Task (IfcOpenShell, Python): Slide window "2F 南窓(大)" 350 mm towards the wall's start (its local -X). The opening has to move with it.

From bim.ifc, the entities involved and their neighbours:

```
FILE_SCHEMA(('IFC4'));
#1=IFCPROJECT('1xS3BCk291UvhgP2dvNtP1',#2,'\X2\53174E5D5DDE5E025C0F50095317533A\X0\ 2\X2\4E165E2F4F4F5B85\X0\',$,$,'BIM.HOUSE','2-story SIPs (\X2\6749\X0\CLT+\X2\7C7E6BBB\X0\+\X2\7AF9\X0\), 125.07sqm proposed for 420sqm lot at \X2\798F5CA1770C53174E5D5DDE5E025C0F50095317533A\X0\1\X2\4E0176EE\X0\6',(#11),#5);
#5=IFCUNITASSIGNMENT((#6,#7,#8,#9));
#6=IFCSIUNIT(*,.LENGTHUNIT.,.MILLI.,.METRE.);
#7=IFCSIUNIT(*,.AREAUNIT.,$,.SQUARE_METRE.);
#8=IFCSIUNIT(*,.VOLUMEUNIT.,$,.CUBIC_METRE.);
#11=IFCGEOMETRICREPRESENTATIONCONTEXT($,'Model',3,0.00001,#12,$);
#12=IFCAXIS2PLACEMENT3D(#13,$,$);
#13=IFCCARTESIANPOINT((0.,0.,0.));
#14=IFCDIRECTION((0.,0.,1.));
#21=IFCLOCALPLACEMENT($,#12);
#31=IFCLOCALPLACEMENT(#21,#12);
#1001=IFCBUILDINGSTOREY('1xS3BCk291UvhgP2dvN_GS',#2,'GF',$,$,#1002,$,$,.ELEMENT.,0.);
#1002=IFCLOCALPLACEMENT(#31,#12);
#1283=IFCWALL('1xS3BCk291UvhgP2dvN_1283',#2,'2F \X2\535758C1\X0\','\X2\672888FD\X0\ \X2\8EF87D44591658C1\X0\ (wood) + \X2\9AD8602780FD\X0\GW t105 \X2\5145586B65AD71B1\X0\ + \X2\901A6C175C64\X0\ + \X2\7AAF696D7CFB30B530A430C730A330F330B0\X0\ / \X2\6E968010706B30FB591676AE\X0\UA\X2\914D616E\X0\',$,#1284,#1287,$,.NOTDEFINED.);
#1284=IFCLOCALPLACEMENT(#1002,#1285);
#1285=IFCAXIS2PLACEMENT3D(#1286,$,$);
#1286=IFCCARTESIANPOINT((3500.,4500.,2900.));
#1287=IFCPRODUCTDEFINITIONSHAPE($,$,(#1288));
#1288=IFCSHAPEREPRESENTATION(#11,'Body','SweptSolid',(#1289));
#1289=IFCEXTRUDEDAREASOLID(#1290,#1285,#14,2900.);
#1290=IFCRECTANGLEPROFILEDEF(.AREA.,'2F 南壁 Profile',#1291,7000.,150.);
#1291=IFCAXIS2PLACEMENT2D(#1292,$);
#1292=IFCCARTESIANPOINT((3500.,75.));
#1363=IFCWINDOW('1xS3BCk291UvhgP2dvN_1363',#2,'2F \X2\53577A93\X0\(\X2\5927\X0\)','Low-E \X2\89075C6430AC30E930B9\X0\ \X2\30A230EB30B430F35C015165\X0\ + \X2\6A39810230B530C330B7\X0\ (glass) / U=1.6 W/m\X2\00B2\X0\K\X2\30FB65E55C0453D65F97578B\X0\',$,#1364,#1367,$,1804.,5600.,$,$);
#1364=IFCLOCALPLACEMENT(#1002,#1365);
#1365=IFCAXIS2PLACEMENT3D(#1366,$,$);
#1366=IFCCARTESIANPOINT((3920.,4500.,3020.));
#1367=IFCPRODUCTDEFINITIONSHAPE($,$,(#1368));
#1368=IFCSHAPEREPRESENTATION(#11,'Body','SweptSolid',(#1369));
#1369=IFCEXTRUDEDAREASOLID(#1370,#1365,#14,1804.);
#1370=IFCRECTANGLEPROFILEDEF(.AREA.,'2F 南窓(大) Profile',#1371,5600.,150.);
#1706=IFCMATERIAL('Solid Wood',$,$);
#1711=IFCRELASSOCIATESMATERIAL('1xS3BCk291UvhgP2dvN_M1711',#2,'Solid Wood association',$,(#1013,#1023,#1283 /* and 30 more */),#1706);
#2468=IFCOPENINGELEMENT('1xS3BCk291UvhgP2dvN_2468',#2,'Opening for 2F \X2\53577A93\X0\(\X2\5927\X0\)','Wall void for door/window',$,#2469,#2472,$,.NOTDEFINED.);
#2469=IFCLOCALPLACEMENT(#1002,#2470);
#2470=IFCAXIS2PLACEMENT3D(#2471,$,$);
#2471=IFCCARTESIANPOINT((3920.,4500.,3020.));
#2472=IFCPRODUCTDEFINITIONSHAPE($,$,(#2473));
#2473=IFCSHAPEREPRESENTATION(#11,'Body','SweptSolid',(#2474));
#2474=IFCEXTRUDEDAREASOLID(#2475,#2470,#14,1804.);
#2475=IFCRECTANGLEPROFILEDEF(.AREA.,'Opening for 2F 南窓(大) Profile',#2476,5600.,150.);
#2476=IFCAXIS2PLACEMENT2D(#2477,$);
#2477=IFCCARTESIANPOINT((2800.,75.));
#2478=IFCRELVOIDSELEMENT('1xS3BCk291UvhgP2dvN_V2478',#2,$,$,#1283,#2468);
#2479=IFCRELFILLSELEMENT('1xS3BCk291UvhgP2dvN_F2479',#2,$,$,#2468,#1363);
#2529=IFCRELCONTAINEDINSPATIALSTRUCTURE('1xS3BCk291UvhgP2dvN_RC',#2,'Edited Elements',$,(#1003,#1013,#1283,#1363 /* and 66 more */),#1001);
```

```python
import ifcopenshell
import ifcopenshell.api.geometry
import ifcopenshell.util.placement
import ifcopenshell.util.unit

model = ifcopenshell.open("bim.ifc")
unit_scale = ifcopenshell.util.unit.calculate_unit_scale(model)

window = model.by_id(1363)
opening = window.FillsVoids[0].RelatingOpeningElement
wall = opening.VoidsElements[0].RelatingBuildingElement

wall_matrix = ifcopenshell.util.placement.get_local_placement(wall.ObjectPlacement)
shift = wall_matrix[:3, 0] * -0.35 / unit_scale
before = ifcopenshell.util.placement.get_local_placement(window.ObjectPlacement)[:3, 3].copy()

# The window is not placed relative to its opening, so move both.
for product in (opening, window):
    matrix = ifcopenshell.util.placement.get_local_placement(product.ObjectPlacement)
    matrix[:3, 3] += shift
    ifcopenshell.api.geometry.edit_object_placement(model, product=product, matrix=matrix, is_si=False)

after = ifcopenshell.util.placement.get_local_placement(window.ObjectPlacement)[:3, 3]
print("window moved by", (after - before).round(3) + 0.0)

model.write("bim_edited.ifc")
```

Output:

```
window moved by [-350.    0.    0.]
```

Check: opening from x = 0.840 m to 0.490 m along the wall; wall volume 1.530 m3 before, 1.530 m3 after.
